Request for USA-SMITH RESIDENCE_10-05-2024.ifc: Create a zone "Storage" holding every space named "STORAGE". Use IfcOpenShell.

First a look at what the model holds.

```python
import ifcopenshell

model = ifcopenshell.open("USA-SMITH RESIDENCE_10-05-2024.ifc")
print(model.schema)
seen = {}
for space in model.by_type("IfcSpace"):
    seen[space.LongName] = seen.get(space.LongName, 0) + 1
for name, count in sorted(seen.items(), key=str):
    print(count, "x", name)
print("zones:", [z.Name for z in model.by_type("IfcZone")][:20])
```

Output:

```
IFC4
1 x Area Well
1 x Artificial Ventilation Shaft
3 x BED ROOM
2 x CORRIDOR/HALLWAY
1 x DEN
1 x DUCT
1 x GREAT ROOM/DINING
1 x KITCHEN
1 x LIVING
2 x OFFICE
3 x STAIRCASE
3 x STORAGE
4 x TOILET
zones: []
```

```python
import ifcopenshell
import ifcopenshell.api.group
import ifcopenshell.api.root

model = ifcopenshell.open("USA-SMITH RESIDENCE_10-05-2024.ifc")

names = {"STORAGE"}
spaces = [s for s in model.by_type("IfcSpace") if s.LongName in names]

zone = ifcopenshell.api.root.create_entity(model, ifc_class="IfcZone", name="Storage")
ifcopenshell.api.group.assign_group(model, products=spaces, group=zone)
print(len(spaces), "spaces in", zone.Name)

model.write("USA-SMITH RESIDENCE_10-05-2024_v2.ifc")
```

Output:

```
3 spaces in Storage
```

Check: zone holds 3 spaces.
